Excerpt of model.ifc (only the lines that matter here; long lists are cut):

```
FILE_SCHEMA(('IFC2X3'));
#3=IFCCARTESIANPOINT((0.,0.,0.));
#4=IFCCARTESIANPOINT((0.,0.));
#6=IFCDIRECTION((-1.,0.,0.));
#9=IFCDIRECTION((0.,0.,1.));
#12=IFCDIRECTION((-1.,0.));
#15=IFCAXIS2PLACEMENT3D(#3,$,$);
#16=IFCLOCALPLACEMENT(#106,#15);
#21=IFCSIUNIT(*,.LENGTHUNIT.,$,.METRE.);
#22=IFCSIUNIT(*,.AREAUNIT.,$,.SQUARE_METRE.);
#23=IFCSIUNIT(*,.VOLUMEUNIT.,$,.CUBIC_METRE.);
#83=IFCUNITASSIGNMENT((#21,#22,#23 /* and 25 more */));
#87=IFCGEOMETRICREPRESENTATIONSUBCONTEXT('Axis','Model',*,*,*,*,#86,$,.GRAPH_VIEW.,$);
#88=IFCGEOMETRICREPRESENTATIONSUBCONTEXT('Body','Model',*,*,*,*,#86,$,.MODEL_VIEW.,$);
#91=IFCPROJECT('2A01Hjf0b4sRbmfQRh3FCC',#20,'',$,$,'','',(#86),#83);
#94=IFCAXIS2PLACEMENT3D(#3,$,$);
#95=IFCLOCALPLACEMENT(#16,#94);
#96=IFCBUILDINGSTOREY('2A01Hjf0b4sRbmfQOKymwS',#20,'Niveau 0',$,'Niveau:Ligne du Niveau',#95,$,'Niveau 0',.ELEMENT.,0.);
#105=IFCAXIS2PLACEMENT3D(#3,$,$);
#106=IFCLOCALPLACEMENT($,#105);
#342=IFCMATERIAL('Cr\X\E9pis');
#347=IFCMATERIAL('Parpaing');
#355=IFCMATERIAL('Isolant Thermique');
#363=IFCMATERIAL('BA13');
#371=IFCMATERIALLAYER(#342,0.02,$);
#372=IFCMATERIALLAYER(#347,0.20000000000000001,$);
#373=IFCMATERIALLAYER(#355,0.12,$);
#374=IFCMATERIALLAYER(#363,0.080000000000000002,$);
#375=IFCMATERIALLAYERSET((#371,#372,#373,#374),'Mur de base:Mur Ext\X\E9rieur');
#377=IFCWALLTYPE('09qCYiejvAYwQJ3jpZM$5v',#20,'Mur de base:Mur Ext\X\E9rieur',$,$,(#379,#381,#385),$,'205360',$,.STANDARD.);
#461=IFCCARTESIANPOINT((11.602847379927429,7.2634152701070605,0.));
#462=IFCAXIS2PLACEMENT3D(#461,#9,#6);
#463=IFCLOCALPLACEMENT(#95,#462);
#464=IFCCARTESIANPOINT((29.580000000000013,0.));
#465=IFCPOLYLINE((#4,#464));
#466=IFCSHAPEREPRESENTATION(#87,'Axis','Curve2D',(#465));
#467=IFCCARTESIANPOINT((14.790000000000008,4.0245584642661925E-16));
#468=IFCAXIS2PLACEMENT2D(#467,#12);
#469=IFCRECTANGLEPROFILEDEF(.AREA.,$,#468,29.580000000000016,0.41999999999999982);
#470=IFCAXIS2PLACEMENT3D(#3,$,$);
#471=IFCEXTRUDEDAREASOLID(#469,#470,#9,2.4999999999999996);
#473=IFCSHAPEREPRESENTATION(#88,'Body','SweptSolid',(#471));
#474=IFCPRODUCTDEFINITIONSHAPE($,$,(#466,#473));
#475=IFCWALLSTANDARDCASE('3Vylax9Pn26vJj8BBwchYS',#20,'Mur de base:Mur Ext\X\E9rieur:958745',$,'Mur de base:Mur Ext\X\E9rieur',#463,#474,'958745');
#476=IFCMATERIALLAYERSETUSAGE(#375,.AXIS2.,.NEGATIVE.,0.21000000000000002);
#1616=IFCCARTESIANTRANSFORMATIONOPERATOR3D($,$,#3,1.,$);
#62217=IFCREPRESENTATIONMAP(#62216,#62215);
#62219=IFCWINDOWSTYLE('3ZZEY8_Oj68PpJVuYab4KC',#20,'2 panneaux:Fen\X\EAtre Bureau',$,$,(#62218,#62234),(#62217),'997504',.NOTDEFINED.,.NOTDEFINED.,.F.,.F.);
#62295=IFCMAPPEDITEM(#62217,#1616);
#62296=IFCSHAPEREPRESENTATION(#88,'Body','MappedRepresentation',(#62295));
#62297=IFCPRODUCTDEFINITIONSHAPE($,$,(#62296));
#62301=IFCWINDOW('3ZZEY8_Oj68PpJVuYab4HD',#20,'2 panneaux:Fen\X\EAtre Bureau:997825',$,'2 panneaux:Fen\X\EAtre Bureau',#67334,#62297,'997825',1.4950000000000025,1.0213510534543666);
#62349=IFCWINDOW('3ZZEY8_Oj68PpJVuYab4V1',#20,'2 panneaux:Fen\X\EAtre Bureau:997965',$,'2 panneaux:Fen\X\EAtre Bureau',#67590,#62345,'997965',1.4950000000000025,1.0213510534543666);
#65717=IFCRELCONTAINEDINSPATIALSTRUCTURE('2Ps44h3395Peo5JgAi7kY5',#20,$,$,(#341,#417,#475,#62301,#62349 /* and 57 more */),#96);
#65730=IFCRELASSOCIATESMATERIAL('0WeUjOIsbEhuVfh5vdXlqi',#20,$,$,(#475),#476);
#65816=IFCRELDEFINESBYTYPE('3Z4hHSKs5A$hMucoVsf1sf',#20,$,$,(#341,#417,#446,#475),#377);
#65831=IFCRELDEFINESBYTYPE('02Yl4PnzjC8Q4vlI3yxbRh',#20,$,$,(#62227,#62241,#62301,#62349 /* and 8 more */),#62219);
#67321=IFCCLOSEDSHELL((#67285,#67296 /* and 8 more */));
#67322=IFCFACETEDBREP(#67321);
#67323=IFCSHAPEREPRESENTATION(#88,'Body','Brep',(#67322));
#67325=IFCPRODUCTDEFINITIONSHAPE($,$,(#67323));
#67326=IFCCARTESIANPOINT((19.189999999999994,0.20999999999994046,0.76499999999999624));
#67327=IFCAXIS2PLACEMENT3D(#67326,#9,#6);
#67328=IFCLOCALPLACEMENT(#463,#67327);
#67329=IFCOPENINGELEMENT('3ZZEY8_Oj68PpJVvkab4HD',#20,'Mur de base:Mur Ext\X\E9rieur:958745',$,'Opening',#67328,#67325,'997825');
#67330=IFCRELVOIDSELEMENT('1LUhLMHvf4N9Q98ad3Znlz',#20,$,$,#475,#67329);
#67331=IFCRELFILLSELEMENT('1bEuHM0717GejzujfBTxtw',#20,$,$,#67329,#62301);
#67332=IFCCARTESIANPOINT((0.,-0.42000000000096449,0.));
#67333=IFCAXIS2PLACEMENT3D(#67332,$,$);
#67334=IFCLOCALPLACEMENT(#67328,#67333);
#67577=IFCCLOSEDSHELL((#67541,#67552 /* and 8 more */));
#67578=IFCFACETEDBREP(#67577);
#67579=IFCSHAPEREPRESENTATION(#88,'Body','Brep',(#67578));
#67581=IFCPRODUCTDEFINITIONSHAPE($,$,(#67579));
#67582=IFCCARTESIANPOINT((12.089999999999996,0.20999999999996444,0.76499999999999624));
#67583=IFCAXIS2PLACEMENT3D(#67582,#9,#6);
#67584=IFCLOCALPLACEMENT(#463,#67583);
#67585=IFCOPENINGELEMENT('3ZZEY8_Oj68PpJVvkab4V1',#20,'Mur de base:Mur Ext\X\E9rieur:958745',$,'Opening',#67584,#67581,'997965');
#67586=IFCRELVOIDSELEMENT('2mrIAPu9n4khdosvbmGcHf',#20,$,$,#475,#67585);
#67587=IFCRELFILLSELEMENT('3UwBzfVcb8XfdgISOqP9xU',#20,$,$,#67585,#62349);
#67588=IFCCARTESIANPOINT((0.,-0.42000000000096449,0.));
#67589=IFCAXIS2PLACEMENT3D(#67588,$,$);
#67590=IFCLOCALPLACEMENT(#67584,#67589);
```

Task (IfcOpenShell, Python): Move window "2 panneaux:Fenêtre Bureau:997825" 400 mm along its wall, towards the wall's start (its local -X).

```python
import ifcopenshell
import ifcopenshell.api.geometry
import ifcopenshell.util.placement

model = ifcopenshell.open("model.ifc")

window = model.by_guid("3ZZEY8_Oj68PpJVuYab4HD")
opening = window.FillsVoids[0].RelatingOpeningElement
wall = opening.VoidsElements[0].RelatingBuildingElement

wall_matrix = ifcopenshell.util.placement.get_local_placement(wall.ObjectPlacement)
shift = wall_matrix[:3, 0] * -0.4
before = ifcopenshell.util.placement.get_local_placement(window.ObjectPlacement)[:3, 3].copy()

# The window is placed relative to its opening, so it follows when the opening moves.
matrix = ifcopenshell.util.placement.get_local_placement(opening.ObjectPlacement)
matrix[:3, 3] += shift
ifcopenshell.api.geometry.edit_object_placement(
    model, product=opening, matrix=matrix, is_si=False, should_transform_children=True
)

after = ifcopenshell.util.placement.get_local_placement(window.ObjectPlacement)[:3, 3]
print("window moved by", (after - before).round(3) + 0.0)

model.write("model_rev.ifc")
```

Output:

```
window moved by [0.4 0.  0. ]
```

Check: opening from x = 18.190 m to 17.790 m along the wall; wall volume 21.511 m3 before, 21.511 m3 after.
